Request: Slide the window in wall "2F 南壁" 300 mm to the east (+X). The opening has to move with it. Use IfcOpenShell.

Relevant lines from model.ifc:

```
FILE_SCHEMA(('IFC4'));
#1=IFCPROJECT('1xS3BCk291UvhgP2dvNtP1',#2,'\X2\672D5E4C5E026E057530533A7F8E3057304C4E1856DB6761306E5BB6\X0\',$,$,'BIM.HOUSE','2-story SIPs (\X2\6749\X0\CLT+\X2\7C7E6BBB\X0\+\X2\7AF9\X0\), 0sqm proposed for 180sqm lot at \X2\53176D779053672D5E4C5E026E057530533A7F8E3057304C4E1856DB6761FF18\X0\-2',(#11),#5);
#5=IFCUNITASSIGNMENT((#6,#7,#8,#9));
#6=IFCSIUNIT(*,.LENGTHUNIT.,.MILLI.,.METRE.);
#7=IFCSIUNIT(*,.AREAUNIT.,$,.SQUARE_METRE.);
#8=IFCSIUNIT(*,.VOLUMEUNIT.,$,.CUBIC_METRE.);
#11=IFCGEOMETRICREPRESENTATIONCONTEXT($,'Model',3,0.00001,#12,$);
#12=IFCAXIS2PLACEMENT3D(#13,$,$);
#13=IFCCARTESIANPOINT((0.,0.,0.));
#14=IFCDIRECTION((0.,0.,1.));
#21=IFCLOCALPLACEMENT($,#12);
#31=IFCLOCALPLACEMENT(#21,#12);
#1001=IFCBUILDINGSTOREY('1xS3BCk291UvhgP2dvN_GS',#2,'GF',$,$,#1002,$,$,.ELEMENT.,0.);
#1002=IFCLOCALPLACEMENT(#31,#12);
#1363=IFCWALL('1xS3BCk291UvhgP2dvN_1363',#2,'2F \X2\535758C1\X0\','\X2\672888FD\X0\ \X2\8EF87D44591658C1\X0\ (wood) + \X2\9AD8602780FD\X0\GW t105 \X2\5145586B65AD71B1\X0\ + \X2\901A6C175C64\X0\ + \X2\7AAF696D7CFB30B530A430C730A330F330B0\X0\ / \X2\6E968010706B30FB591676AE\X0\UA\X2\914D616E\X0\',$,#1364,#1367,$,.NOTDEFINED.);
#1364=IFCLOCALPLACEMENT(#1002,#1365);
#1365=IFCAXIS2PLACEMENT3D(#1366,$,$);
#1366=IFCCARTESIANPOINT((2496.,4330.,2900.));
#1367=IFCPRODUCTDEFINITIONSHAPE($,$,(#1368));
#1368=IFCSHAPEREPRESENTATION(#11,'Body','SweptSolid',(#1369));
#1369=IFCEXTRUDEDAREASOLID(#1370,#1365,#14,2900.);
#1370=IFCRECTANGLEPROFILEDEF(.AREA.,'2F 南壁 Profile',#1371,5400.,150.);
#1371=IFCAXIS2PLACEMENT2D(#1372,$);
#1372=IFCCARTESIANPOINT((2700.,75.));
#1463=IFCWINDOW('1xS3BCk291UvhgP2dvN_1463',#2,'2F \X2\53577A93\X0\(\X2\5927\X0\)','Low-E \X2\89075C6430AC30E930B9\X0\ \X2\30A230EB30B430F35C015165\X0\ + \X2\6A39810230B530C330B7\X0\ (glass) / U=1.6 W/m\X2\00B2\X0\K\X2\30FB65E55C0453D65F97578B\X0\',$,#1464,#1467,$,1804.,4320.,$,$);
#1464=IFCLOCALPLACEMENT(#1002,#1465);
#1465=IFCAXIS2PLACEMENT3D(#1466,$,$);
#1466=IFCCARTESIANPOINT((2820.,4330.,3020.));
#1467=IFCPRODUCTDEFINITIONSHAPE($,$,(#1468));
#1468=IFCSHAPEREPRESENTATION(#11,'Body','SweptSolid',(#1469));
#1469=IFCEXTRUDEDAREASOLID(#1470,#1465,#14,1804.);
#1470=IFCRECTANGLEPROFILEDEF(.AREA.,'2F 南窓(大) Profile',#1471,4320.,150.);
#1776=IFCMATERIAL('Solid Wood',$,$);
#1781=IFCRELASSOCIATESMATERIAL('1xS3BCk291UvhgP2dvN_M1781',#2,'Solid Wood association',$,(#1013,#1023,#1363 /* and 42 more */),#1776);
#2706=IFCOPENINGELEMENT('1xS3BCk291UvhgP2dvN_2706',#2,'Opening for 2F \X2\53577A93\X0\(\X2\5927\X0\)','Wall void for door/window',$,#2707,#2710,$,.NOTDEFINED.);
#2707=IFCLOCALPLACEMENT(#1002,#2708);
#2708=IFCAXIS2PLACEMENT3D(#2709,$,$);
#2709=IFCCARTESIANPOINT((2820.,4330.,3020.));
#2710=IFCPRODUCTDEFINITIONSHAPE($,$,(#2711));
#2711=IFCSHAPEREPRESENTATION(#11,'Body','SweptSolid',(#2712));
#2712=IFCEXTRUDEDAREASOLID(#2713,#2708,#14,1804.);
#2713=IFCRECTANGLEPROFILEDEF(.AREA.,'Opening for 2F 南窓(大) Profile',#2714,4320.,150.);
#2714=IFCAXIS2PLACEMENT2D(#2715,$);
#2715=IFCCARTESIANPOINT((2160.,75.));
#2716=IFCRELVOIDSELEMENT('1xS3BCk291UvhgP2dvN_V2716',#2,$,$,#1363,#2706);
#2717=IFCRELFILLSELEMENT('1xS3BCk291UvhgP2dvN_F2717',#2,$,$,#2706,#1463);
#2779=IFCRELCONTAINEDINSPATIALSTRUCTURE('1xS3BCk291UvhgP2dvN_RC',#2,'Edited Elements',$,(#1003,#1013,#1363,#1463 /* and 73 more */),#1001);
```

```python
import ifcopenshell
import ifcopenshell.api.geometry
import ifcopenshell.util.placement

model = ifcopenshell.open("model.ifc")

window = model.by_id(1463)
opening = window.FillsVoids[0].RelatingOpeningElement
wall = opening.VoidsElements[0].RelatingBuildingElement

wall_matrix = ifcopenshell.util.placement.get_local_placement(wall.ObjectPlacement)
shift = wall_matrix[:3, 0] * 300.0
before = ifcopenshell.util.placement.get_local_placement(window.ObjectPlacement)[:3, 3].copy()

# The window is not placed relative to its opening, so move both.
for product in (opening, window):
    matrix = ifcopenshell.util.placement.get_local_placement(product.ObjectPlacement)
    matrix[:3, 3] += shift
    ifcopenshell.api.geometry.edit_object_placement(model, product=product, matrix=matrix, is_si=False)

after = ifcopenshell.util.placement.get_local_placement(window.ObjectPlacement)[:3, 3]
print("window moved by", (after - before).round(3) + 0.0)

model.write("model_rev.ifc")
```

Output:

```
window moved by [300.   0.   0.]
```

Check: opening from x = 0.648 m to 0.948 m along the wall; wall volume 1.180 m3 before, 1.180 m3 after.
